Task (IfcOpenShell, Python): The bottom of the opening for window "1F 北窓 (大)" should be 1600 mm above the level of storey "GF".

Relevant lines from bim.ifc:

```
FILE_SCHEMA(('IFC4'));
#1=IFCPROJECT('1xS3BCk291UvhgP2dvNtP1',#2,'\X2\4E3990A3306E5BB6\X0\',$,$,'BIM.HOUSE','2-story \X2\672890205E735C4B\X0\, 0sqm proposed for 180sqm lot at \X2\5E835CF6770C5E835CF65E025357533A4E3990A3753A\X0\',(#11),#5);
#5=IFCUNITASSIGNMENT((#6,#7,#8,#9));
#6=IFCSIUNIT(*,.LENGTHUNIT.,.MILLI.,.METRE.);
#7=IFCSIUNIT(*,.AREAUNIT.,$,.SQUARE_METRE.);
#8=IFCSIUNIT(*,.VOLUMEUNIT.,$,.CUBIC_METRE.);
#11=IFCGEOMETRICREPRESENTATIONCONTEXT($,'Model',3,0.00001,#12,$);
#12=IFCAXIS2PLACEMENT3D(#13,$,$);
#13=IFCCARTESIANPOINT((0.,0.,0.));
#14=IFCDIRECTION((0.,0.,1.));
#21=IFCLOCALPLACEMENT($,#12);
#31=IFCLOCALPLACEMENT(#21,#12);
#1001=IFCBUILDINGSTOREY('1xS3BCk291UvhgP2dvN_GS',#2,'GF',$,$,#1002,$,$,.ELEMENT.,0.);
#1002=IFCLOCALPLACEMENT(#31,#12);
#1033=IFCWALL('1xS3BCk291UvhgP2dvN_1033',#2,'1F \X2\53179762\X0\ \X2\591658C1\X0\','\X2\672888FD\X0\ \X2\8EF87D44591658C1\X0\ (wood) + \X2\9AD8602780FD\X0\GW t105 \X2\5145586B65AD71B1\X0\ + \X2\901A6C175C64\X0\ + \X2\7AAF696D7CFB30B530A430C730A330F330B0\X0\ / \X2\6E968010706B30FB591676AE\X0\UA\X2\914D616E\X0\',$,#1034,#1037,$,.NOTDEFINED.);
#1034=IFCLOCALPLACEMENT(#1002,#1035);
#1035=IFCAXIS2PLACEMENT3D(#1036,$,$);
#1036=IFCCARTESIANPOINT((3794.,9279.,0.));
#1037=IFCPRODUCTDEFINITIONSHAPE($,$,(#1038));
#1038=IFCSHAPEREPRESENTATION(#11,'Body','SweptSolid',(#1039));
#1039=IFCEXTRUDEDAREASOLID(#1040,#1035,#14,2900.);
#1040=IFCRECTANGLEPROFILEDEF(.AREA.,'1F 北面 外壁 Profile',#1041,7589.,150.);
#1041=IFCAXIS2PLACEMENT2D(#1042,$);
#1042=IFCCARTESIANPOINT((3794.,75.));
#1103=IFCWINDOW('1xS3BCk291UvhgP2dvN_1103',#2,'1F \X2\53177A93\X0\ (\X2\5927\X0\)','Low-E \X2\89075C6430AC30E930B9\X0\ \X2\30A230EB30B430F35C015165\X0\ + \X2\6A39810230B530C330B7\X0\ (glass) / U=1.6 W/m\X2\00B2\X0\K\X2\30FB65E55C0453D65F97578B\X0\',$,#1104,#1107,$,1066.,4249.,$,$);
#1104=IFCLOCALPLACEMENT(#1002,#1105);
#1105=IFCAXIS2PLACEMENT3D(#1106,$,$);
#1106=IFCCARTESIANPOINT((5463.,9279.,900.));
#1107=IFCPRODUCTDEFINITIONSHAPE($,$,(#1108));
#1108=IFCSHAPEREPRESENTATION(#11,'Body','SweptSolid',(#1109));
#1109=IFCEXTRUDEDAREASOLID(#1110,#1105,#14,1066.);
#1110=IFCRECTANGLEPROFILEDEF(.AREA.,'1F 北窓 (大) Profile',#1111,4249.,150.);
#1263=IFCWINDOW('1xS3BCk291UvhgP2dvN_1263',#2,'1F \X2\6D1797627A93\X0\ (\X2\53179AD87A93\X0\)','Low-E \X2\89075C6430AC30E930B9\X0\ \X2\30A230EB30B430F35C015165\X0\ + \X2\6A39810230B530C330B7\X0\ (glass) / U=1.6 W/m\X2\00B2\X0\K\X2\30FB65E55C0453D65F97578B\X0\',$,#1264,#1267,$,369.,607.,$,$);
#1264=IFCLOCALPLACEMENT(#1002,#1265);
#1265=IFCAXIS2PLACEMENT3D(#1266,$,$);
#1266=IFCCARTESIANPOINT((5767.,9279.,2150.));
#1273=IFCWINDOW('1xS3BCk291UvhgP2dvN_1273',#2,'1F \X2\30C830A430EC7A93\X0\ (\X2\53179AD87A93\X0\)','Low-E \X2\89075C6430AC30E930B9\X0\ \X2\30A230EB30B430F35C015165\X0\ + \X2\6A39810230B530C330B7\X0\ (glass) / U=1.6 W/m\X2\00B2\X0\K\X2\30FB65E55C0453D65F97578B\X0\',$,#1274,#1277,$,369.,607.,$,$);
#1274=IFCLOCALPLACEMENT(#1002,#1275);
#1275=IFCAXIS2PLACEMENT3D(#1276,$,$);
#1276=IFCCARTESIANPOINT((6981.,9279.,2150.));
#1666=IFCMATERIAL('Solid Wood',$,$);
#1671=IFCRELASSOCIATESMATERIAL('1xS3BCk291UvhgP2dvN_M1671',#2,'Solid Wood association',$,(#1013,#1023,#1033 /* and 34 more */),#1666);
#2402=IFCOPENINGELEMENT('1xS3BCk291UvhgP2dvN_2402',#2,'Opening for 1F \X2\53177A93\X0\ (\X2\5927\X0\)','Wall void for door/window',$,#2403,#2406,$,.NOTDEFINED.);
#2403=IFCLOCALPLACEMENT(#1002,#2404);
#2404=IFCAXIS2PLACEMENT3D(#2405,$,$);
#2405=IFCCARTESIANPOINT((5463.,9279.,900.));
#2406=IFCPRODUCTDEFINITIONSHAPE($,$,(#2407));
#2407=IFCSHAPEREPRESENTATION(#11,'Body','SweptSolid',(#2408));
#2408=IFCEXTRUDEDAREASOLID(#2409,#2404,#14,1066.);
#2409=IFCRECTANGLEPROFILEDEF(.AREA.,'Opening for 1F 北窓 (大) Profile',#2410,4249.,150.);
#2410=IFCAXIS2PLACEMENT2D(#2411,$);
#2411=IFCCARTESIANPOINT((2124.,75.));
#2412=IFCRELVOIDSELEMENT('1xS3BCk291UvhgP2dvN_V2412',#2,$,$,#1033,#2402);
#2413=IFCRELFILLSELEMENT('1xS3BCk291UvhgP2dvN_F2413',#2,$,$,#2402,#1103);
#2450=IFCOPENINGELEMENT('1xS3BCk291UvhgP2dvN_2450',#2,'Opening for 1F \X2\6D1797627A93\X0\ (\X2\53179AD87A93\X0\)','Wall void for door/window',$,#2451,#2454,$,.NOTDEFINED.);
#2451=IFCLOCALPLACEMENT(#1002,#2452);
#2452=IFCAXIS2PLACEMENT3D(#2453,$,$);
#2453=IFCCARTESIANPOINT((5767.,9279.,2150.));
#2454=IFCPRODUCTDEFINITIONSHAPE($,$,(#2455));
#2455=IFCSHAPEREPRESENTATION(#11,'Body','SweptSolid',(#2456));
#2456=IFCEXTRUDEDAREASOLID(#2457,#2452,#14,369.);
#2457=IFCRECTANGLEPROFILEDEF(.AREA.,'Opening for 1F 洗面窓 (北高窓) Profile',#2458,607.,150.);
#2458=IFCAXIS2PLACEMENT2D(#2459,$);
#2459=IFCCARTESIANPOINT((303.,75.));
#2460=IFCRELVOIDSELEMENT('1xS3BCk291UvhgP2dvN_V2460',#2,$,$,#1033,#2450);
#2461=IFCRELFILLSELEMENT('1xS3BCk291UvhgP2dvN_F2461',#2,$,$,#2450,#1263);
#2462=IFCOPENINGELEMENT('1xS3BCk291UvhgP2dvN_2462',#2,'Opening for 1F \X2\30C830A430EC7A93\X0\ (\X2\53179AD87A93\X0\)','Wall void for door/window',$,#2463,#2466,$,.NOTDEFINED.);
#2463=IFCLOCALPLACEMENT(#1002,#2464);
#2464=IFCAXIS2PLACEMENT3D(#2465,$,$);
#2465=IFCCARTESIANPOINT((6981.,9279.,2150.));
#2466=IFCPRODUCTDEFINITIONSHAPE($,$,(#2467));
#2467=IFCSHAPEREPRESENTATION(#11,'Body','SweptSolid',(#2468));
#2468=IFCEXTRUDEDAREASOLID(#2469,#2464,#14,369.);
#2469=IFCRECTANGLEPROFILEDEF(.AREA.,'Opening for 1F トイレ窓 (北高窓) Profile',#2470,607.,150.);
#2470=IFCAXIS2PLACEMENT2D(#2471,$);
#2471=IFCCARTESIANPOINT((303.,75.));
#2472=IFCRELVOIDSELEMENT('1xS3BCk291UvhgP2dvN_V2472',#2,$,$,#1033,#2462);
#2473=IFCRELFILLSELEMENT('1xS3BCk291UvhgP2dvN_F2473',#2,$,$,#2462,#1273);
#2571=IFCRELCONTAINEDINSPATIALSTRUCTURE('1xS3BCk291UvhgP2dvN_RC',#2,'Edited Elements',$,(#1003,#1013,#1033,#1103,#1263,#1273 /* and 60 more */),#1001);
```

```python
import numpy as np
import ifcopenshell
import ifcopenshell.api.geometry
import ifcopenshell.geom
import ifcopenshell.util.element
import ifcopenshell.util.placement
import ifcopenshell.util.shape
import ifcopenshell.util.unit

model = ifcopenshell.open("bim.ifc")
unit_scale = ifcopenshell.util.unit.calculate_unit_scale(model)

window = model.by_guid("1xS3BCk291UvhgP2dvN_1103")
opening = window.FillsVoids[0].RelatingOpeningElement
storey = ifcopenshell.util.element.get_container(window, ifc_class="IfcBuildingStorey")
level = ifcopenshell.util.placement.get_local_placement(storey.ObjectPlacement)[2, 3]

# The opening's origin need not be at the sill, so measure its lowest point.
shape = ifcopenshell.geom.create_shape(ifcopenshell.geom.settings(), opening)
bottom = ifcopenshell.util.shape.get_shape_bottom_elevation(shape, shape.geometry) / unit_scale
dz = level + 1.6 / unit_scale - bottom

shift = np.array([0.0, 0.0, dz])
# The window is not placed relative to its opening, so move both.
for product in (opening, window):
    matrix = ifcopenshell.util.placement.get_local_placement(product.ObjectPlacement)
    matrix[:3, 3] += shift
    ifcopenshell.api.geometry.edit_object_placement(model, product=product, matrix=matrix, is_si=False)

print(f"moved by {dz * unit_scale:+.3f} m")

model.write("bim_v2.ifc")
```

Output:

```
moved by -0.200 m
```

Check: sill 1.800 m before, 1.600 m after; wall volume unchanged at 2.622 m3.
